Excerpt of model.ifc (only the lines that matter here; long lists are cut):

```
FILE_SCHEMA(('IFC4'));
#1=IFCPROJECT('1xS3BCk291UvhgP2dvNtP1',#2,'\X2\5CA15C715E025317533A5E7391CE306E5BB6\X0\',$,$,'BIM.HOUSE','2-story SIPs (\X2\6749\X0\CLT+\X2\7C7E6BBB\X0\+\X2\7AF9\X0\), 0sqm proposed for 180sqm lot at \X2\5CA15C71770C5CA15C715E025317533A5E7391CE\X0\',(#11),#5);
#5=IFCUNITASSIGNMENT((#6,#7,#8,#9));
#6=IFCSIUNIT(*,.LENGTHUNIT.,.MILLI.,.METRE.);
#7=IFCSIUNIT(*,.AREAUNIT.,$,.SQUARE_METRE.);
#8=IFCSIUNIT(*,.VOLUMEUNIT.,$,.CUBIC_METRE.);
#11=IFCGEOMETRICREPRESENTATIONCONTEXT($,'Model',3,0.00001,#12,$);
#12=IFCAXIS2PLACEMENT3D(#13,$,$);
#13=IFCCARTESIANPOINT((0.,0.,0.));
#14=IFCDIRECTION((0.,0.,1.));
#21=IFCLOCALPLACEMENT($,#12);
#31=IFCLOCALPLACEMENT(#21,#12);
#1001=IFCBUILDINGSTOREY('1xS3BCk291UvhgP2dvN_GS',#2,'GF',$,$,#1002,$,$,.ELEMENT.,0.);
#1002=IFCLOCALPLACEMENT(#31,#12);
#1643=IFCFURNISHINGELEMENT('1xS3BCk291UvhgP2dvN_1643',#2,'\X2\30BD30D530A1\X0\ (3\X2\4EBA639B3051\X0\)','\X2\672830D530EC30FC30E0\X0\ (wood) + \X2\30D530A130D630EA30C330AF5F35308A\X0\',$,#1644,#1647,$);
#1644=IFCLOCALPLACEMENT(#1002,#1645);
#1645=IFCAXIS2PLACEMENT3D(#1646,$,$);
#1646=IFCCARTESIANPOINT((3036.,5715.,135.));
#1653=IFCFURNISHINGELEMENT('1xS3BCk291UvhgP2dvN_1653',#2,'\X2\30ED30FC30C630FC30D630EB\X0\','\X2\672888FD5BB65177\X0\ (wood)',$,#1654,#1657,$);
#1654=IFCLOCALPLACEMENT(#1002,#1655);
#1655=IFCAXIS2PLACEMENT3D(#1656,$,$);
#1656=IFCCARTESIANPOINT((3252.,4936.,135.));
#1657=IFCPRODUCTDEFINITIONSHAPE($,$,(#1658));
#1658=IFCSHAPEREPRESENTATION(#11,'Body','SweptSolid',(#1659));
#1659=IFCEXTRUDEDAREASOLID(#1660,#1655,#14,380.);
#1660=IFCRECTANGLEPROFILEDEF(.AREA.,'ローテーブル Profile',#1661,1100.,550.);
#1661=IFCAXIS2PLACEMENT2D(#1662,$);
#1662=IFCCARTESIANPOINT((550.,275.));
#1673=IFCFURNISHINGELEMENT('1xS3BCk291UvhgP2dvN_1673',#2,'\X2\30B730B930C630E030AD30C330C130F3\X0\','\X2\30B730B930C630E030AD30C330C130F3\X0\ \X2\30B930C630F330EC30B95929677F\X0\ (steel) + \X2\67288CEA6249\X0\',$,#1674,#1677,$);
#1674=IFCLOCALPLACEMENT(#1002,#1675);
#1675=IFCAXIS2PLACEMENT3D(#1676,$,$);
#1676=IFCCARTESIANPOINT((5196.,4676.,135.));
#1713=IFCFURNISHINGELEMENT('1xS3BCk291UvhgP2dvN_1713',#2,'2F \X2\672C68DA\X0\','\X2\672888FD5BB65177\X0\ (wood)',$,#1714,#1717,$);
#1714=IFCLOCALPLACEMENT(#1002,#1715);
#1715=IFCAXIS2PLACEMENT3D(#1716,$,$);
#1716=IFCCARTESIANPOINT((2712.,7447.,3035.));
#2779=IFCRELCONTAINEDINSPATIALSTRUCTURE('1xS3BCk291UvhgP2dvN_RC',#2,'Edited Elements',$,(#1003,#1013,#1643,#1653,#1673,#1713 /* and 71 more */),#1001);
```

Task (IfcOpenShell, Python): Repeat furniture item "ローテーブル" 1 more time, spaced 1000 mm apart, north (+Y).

```python
import numpy as np
import ifcopenshell
import ifcopenshell.api.geometry
import ifcopenshell.api.root
import ifcopenshell.util.element
import ifcopenshell.util.placement
import ifcopenshell.util.unit

model = ifcopenshell.open("model.ifc")
unit_scale = ifcopenshell.util.unit.calculate_unit_scale(model)


def reuse_history(source, copy):
    """copy_class also copies each property set's owner history, people and application; keep the originals."""
    for rel in copy.IsDefinedBy:
        if rel.is_a("IfcRelDefinesByProperties") and (history := rel.RelatingPropertyDefinition.OwnerHistory):
            rel.RelatingPropertyDefinition.OwnerHistory = source.OwnerHistory
            ifcopenshell.util.element.remove_deep2(model, history)


source = model.by_id(1653)
base = ifcopenshell.util.placement.get_local_placement(source.ObjectPlacement)
step = np.array([0.0, 1.0, 0.0]) * 1 / unit_scale

for i in range(1, 2):
    copy = ifcopenshell.api.root.copy_class(model, product=source)
    copy.Representation = ifcopenshell.util.element.copy_deep(
        model, source.Representation, exclude=["IfcGeometricRepresentationContext", "IfcRepresentationMap"]
    )
    reuse_history(source, copy)
    matrix = base.copy()
    matrix[:3, 3] += i * step
    print("added at", matrix[:3, 3].round(3) + 0.0)
    ifcopenshell.api.geometry.edit_object_placement(model, product=copy, matrix=matrix, is_si=False)

model.write("model_updated.ifc")
```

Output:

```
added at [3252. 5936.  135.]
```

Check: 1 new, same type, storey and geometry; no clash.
